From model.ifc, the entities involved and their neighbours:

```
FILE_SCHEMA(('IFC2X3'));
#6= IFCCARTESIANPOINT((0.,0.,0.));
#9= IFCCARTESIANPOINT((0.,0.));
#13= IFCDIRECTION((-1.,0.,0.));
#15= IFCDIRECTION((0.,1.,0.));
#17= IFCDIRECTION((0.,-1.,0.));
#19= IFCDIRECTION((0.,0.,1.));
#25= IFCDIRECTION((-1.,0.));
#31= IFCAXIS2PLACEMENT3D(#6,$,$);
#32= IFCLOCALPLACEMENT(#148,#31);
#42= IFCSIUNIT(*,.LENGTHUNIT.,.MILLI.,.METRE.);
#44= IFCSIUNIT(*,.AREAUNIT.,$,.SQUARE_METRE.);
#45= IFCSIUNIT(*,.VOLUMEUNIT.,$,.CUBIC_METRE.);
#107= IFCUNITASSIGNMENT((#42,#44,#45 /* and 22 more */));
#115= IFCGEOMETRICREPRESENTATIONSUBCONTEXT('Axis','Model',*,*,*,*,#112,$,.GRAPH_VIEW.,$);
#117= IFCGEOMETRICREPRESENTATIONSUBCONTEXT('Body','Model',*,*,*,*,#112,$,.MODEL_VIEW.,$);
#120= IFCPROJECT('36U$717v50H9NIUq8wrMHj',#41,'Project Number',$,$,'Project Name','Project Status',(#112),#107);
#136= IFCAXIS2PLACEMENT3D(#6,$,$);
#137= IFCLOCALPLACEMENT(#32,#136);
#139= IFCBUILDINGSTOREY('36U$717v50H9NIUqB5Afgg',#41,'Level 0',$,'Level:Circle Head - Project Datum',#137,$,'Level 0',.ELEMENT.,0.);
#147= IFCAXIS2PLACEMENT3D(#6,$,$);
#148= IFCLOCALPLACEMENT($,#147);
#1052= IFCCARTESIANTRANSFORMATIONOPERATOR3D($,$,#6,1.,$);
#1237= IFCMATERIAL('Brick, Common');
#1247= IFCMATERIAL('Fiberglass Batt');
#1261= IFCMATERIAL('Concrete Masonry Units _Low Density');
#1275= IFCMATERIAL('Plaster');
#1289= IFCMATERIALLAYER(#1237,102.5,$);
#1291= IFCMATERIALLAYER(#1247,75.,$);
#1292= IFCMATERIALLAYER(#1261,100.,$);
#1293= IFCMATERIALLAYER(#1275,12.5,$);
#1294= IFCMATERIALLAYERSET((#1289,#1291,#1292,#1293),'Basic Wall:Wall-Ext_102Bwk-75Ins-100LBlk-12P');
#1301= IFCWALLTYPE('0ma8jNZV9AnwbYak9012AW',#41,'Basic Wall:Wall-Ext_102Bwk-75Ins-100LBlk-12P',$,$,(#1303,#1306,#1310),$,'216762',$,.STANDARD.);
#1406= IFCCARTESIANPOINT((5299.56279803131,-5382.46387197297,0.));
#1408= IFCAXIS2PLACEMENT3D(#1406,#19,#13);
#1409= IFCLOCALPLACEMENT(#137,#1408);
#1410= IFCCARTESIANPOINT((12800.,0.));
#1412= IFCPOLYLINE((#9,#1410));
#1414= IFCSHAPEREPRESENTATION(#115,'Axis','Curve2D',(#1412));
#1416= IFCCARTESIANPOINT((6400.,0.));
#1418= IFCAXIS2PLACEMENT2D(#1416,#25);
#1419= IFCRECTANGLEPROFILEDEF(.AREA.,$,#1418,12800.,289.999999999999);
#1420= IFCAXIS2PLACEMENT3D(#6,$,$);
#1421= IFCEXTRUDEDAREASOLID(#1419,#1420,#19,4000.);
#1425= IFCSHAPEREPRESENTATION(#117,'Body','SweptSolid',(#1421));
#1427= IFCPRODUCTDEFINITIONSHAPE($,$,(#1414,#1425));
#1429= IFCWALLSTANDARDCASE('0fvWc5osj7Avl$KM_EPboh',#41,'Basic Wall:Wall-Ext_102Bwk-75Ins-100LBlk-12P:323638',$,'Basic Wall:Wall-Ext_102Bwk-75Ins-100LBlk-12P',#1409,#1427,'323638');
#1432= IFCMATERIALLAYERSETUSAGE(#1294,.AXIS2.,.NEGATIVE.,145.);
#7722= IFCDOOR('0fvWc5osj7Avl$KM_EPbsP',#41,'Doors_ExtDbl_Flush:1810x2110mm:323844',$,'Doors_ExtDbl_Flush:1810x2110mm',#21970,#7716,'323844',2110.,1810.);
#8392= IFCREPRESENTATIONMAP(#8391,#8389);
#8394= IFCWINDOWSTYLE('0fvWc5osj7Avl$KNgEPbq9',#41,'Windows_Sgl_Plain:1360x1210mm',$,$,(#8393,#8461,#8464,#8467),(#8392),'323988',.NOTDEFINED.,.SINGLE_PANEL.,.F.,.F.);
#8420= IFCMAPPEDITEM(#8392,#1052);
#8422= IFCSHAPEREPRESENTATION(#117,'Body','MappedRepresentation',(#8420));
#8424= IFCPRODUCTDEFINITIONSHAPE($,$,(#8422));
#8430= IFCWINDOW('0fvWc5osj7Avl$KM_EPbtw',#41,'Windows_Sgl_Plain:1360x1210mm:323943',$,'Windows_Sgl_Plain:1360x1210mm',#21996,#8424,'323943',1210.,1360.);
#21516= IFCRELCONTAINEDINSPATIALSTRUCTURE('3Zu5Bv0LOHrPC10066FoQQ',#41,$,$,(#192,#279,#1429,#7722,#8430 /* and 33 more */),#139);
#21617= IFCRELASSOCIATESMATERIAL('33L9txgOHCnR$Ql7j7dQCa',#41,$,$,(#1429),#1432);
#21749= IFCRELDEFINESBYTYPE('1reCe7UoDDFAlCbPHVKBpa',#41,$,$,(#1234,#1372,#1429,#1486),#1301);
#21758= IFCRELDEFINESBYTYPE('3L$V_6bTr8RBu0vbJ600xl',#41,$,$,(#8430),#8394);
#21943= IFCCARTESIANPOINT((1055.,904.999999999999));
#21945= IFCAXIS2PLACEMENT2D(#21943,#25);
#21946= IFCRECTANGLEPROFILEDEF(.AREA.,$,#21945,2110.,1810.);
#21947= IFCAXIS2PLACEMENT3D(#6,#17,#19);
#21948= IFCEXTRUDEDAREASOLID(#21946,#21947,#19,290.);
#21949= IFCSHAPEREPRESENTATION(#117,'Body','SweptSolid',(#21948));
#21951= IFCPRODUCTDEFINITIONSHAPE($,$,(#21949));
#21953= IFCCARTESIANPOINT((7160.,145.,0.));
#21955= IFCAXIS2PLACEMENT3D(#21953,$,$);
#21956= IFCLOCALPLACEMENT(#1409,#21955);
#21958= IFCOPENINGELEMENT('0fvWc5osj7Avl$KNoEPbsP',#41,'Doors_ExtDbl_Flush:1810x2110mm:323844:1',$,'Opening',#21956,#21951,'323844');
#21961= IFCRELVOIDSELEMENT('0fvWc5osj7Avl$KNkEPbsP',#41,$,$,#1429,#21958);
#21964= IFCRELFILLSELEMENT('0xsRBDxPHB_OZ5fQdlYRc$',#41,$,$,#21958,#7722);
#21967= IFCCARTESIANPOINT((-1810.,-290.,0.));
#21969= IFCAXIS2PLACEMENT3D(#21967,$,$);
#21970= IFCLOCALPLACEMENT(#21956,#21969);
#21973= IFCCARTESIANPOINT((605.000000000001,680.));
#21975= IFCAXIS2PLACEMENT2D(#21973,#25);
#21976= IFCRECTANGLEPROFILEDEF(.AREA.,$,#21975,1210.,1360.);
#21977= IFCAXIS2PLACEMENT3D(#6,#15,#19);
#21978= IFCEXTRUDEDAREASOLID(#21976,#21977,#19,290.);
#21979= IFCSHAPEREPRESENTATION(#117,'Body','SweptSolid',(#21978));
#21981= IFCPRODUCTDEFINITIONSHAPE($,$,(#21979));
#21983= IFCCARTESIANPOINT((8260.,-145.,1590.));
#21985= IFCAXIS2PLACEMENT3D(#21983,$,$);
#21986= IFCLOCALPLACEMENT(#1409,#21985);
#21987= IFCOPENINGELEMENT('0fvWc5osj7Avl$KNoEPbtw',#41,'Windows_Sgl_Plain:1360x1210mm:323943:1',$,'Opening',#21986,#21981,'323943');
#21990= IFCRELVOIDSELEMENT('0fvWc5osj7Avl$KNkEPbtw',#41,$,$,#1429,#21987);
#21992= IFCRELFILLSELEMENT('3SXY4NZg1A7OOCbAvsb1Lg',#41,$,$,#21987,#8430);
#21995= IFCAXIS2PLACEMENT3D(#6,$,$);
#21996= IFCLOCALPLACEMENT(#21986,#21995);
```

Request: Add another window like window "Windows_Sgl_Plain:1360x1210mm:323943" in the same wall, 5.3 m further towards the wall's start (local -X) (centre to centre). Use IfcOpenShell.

```python
import ifcopenshell
import ifcopenshell.api.feature
import ifcopenshell.api.geometry
import ifcopenshell.api.root
import ifcopenshell.geom
import ifcopenshell.util.element
import ifcopenshell.util.placement
import ifcopenshell.util.shape
import ifcopenshell.util.unit

model = ifcopenshell.open("model.ifc")
unit_scale = ifcopenshell.util.unit.calculate_unit_scale(model)
settings = ifcopenshell.geom.settings()


def volume(element):
    """Net volume in cubic metres, openings subtracted."""
    shape = ifcopenshell.geom.create_shape(settings, element)
    return ifcopenshell.util.shape.get_volume(shape.geometry)


def reuse_history(source, copy):
    """copy_class also copies each property set's owner history, people and application; keep the originals."""
    for rel in copy.IsDefinedBy:
        if rel.is_a("IfcRelDefinesByProperties") and (history := rel.RelatingPropertyDefinition.OwnerHistory):
            rel.RelatingPropertyDefinition.OwnerHistory = source.OwnerHistory
            ifcopenshell.util.element.remove_deep2(model, history)


window = model.by_id(8430)
opening = window.FillsVoids[0].RelatingOpeningElement
wall = opening.VoidsElements[0].RelatingBuildingElement
before = volume(wall)
shift = ifcopenshell.util.placement.get_local_placement(wall.ObjectPlacement)[:3, 0] * -5.3 / unit_scale

# copy_class copies the void relationship, type, container and properties, but no geometry.
new_opening = ifcopenshell.api.root.copy_class(model, product=opening)
new_opening.Representation = ifcopenshell.util.element.copy_deep(
    model, opening.Representation, exclude=["IfcGeometricRepresentationContext", "IfcRepresentationMap"]
)
new_opening.Name = "Windows_Sgl_Plain:1360x1210mm"
new_opening.Tag = None
new_window = ifcopenshell.api.root.copy_class(model, product=window)
new_window.Representation = ifcopenshell.util.element.copy_deep(
    model, window.Representation, exclude=["IfcGeometricRepresentationContext", "IfcRepresentationMap"]
)
new_window.Name = "Windows_Sgl_Plain:1360x1210mm"
new_window.Tag = None
reuse_history(window, new_window)
fills = ifcopenshell.api.feature.add_filling(model, opening=new_opening, element=new_window)
fills.OwnerHistory = new_window.OwnerHistory  # required in IFC2X3

for old, new in ((opening, new_opening), (window, new_window)):
    matrix = ifcopenshell.util.placement.get_local_placement(old.ObjectPlacement)
    matrix[:3, 3] += shift
    ifcopenshell.api.geometry.edit_object_placement(model, product=new, matrix=matrix, is_si=False)

after = volume(wall)

print(f"wall volume {before:.3f} -> {after:.3f} m3")

model.write("model_v2.ifc")
```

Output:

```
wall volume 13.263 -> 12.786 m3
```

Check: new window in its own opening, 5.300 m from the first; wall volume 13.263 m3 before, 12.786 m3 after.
